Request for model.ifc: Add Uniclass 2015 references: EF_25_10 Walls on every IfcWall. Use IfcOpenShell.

First a look at what the model holds.

```python
import ifcopenshell

model = ifcopenshell.open("model.ifc")
print(model.schema)
print("classifications:", [c.Name for c in model.by_type("IfcClassification")])
for ifc_class in ("IfcDoor", "IfcRoof", "IfcStair", "IfcWall", "IfcWindow"):
    print(ifc_class, len(model.by_type(ifc_class)))
```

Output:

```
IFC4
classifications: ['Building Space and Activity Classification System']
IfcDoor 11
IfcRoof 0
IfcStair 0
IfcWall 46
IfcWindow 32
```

```python
import ifcopenshell
import ifcopenshell.api.classification

model = ifcopenshell.open("model.ifc")

system = ifcopenshell.api.classification.add_classification(model, classification="Uniclass 2015")

codes = {
    "IfcWall": ("EF_25_10", "Walls"),
}
for ifc_class, (code, name) in codes.items():
    products = model.by_type(ifc_class)
    ifcopenshell.api.classification.add_reference(
        model, products=products, classification=system, identification=code, name=name
    )
    print(code, len(products))

model.write("model_rev.ifc")
```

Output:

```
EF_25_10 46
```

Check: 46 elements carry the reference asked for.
